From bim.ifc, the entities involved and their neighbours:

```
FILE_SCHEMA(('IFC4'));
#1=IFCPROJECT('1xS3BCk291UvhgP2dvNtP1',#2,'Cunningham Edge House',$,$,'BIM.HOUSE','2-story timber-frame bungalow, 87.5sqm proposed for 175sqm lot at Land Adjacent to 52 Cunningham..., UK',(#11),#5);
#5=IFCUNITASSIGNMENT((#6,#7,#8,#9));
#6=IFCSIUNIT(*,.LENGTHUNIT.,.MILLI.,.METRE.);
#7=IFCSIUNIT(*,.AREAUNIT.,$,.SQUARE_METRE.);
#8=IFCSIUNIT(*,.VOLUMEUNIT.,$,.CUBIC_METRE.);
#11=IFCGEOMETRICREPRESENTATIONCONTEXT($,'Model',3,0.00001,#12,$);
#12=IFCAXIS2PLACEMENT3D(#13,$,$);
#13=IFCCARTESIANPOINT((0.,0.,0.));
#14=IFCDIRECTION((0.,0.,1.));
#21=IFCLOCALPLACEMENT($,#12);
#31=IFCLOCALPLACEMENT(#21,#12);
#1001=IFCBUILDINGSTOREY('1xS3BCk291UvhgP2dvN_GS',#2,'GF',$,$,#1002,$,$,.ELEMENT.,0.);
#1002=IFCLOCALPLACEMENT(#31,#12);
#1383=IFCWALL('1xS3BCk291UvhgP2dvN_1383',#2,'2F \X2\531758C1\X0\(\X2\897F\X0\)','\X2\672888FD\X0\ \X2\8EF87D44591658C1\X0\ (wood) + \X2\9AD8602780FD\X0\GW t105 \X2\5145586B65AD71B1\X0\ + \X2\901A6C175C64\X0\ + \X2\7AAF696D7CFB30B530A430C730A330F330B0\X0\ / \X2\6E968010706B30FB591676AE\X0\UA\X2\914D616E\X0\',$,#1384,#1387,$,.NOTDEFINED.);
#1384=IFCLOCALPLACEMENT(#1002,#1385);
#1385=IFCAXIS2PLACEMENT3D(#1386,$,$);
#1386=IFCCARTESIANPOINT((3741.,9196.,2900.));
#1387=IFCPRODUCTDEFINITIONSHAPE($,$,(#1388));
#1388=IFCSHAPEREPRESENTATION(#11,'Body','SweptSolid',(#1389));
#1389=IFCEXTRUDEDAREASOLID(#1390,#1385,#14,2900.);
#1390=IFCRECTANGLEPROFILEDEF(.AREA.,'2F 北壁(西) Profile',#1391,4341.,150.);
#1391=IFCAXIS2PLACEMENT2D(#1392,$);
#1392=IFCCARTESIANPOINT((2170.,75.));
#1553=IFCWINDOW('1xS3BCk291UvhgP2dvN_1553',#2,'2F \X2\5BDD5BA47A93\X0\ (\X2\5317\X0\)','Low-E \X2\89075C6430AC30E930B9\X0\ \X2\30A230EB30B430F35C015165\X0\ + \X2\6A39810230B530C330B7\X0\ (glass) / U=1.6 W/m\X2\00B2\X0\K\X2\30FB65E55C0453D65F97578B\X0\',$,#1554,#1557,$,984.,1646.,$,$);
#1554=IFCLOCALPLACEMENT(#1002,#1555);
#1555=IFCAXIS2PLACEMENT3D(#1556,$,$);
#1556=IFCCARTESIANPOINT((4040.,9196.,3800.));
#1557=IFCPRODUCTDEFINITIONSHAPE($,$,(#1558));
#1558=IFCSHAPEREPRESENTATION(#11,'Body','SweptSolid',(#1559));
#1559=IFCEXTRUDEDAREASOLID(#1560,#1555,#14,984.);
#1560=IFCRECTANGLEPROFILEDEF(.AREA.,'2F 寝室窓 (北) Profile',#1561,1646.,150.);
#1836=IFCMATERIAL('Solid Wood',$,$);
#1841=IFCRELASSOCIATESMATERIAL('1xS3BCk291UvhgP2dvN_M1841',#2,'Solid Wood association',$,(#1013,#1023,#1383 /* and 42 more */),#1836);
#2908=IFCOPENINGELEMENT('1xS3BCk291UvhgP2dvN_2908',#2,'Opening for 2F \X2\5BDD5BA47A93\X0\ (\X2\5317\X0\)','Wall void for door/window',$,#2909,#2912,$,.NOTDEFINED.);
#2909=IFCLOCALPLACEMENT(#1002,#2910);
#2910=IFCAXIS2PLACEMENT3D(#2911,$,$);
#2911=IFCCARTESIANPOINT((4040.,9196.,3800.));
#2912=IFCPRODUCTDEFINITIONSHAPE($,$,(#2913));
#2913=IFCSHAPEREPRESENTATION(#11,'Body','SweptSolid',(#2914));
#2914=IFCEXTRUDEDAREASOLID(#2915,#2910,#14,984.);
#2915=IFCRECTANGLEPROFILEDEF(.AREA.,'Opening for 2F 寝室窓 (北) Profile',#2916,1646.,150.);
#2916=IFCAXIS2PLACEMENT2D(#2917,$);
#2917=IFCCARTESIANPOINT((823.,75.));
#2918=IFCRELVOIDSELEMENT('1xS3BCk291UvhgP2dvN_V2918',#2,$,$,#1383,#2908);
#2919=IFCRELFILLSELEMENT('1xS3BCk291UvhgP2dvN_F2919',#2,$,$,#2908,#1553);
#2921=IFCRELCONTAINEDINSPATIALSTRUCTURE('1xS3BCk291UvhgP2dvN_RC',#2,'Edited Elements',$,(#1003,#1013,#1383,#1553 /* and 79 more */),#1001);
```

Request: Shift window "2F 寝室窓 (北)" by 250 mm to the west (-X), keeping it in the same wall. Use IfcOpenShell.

```python
import ifcopenshell
import ifcopenshell.api.geometry
import ifcopenshell.util.placement

model = ifcopenshell.open("bim.ifc")

window = model.by_guid("1xS3BCk291UvhgP2dvN_1553")
opening = window.FillsVoids[0].RelatingOpeningElement
wall = opening.VoidsElements[0].RelatingBuildingElement

wall_matrix = ifcopenshell.util.placement.get_local_placement(wall.ObjectPlacement)
shift = wall_matrix[:3, 0] * -250.0
before = ifcopenshell.util.placement.get_local_placement(window.ObjectPlacement)[:3, 3].copy()

# The window is not placed relative to its opening, so move both.
for product in (opening, window):
    matrix = ifcopenshell.util.placement.get_local_placement(product.ObjectPlacement)
    matrix[:3, 3] += shift
    ifcopenshell.api.geometry.edit_object_placement(model, product=product, matrix=matrix, is_si=False)

after = ifcopenshell.util.placement.get_local_placement(window.ObjectPlacement)[:3, 3]
print("window moved by", (after - before).round(3) + 0.0)

model.write("bim_rev.ifc")
```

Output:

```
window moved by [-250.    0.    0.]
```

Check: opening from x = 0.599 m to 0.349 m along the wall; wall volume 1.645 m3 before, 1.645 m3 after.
